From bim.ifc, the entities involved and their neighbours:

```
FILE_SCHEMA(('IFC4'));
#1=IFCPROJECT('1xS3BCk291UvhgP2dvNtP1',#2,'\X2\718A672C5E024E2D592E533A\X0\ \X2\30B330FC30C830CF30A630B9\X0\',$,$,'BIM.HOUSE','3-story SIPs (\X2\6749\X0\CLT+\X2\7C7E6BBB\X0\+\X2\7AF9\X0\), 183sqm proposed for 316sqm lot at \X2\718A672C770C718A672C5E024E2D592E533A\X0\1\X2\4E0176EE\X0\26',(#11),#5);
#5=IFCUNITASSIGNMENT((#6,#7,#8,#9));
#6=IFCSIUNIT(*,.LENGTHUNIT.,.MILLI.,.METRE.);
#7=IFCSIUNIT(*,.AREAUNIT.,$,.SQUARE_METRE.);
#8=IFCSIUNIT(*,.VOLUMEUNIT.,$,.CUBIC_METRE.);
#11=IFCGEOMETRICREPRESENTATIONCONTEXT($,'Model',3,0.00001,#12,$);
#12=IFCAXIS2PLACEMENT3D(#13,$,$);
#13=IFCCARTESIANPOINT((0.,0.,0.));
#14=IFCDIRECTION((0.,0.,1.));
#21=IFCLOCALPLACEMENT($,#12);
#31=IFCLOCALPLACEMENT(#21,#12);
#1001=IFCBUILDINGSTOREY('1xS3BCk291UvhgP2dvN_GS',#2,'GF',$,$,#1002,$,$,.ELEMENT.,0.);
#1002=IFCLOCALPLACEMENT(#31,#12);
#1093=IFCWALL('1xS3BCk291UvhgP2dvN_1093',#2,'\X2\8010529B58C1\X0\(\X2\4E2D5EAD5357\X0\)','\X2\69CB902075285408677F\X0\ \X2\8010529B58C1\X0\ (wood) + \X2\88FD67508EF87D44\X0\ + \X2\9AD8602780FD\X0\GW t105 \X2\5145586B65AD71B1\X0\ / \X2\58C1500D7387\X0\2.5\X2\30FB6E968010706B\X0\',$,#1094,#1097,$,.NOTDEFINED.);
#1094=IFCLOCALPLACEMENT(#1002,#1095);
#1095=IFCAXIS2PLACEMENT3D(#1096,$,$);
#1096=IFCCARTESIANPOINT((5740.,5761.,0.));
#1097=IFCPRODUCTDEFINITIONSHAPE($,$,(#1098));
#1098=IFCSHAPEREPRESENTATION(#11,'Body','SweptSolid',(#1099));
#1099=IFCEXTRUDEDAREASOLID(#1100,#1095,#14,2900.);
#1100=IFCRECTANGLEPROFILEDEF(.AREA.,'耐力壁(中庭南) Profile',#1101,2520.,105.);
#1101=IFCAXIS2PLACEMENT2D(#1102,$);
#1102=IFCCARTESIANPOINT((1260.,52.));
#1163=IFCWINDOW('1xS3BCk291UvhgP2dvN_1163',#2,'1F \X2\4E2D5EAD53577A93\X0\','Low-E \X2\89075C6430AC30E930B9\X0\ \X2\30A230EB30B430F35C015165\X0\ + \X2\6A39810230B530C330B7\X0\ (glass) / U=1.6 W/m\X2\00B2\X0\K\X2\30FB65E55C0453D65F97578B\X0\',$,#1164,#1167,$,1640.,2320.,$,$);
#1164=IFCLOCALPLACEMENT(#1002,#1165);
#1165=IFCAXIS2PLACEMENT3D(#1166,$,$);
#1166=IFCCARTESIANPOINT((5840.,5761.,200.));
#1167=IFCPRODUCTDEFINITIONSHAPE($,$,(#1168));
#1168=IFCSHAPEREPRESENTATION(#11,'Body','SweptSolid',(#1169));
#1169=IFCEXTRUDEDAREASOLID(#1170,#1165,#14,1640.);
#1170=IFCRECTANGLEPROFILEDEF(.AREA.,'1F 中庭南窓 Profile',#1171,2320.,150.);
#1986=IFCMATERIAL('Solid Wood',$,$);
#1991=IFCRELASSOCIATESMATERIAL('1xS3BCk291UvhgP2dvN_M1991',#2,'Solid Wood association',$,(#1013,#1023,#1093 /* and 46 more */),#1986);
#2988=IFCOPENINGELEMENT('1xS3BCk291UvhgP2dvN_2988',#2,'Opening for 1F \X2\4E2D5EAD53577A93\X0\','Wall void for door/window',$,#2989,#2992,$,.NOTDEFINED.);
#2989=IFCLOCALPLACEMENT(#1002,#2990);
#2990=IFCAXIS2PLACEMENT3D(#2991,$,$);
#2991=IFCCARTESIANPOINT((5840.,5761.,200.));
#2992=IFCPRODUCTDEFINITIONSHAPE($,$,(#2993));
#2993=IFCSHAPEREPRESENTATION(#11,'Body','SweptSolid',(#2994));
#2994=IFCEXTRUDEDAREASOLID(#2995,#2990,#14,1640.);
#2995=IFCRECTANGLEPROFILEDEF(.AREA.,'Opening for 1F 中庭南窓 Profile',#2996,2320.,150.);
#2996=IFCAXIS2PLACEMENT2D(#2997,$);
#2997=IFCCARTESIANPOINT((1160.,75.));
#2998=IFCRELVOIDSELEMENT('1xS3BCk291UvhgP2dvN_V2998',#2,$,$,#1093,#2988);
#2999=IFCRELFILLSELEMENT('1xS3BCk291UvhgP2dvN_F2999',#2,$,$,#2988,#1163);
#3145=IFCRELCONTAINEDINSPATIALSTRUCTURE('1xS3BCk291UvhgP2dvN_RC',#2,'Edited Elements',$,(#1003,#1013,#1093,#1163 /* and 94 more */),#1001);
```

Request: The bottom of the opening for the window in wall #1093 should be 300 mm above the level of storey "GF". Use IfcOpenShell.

```python
import numpy as np
import ifcopenshell
import ifcopenshell.api.geometry
import ifcopenshell.geom
import ifcopenshell.util.element
import ifcopenshell.util.placement
import ifcopenshell.util.shape
import ifcopenshell.util.unit

model = ifcopenshell.open("bim.ifc")
unit_scale = ifcopenshell.util.unit.calculate_unit_scale(model)

window = model.by_id(1163)
opening = window.FillsVoids[0].RelatingOpeningElement
storey = ifcopenshell.util.element.get_container(window, ifc_class="IfcBuildingStorey")
level = ifcopenshell.util.placement.get_local_placement(storey.ObjectPlacement)[2, 3]

# The opening's origin need not be at the sill, so measure its lowest point.
shape = ifcopenshell.geom.create_shape(ifcopenshell.geom.settings(), opening)
bottom = ifcopenshell.util.shape.get_shape_bottom_elevation(shape, shape.geometry) / unit_scale
dz = level + 0.3 / unit_scale - bottom

shift = np.array([0.0, 0.0, dz])
# The window is not placed relative to its opening, so move both.
for product in (opening, window):
    matrix = ifcopenshell.util.placement.get_local_placement(product.ObjectPlacement)
    matrix[:3, 3] += shift
    ifcopenshell.api.geometry.edit_object_placement(model, product=product, matrix=matrix, is_si=False)

print(f"moved by {dz * unit_scale:+.3f} m")

model.write("bim_rev.ifc")
```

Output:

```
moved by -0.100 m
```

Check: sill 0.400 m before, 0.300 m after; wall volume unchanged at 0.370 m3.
